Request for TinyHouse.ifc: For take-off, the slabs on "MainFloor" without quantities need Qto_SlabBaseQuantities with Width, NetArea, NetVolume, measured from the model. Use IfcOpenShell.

First a look at what the model holds.

```python
import ifcopenshell
import ifcopenshell.util.element
import ifcopenshell.util.unit

model = ifcopenshell.open("TinyHouse.ifc")
print(model.schema)
for unit_type in ("LENGTHUNIT", "AREAUNIT", "VOLUMEUNIT"):
    print(unit_type, ifcopenshell.util.unit.calculate_unit_scale(model, unit_type))
storey = next(s for s in model.by_type("IfcBuildingStorey") if s.Name == "MainFloor")
slabs = [e for e in ifcopenshell.util.element.get_decomposition(storey) if e.is_a("IfcSlab")]
for e in sorted(slabs, key=lambda e: e.id()):
    print(e.id(), e.is_a(), e.Name, list(ifcopenshell.util.element.get_psets(e, qtos_only=True)), sep=" | ")
```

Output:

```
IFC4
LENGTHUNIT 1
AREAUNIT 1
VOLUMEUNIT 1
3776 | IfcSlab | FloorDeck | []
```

```python
import ifcopenshell
import ifcopenshell.api.pset
import ifcopenshell.geom
import ifcopenshell.util.element
import ifcopenshell.util.shape
import ifcopenshell.util.unit

model = ifcopenshell.open("TinyHouse.ifc")
unit_scale = ifcopenshell.util.unit.calculate_unit_scale(model)
area_scale = ifcopenshell.util.unit.calculate_unit_scale(model, "AREAUNIT")
volume_scale = ifcopenshell.util.unit.calculate_unit_scale(model, "VOLUMEUNIT")
settings = ifcopenshell.geom.settings()

storey = next(s for s in model.by_type("IfcBuildingStorey") if s.Name == "MainFloor")
slabs = [e for e in ifcopenshell.util.element.get_decomposition(storey) if e.is_a("IfcSlab")]

for e in sorted(slabs, key=lambda e: e.id()):
    if ifcopenshell.util.element.get_psets(e, qtos_only=True, should_inherit=False):
        continue
    # Geometry comes back in metres, in the element's own axes.
    shape = ifcopenshell.geom.create_shape(settings, e)
    values = {
        "Width": ifcopenshell.util.shape.get_z(shape.geometry) / unit_scale,
        "NetArea": ifcopenshell.util.shape.get_footprint_area(shape.geometry) / area_scale,
        "NetVolume": ifcopenshell.util.shape.get_volume(shape.geometry) / volume_scale,
    }
    qto = ifcopenshell.api.pset.add_qto(model, product=e, name="Qto_SlabBaseQuantities")
    ifcopenshell.api.pset.edit_qto(model, qto=qto, properties=values)
    print(e.id(), {k: round(v, 3) for k, v in values.items()})

model.write("TinyHouse_updated.ifc")
```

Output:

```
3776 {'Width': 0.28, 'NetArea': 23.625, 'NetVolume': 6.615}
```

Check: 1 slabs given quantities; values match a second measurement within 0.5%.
